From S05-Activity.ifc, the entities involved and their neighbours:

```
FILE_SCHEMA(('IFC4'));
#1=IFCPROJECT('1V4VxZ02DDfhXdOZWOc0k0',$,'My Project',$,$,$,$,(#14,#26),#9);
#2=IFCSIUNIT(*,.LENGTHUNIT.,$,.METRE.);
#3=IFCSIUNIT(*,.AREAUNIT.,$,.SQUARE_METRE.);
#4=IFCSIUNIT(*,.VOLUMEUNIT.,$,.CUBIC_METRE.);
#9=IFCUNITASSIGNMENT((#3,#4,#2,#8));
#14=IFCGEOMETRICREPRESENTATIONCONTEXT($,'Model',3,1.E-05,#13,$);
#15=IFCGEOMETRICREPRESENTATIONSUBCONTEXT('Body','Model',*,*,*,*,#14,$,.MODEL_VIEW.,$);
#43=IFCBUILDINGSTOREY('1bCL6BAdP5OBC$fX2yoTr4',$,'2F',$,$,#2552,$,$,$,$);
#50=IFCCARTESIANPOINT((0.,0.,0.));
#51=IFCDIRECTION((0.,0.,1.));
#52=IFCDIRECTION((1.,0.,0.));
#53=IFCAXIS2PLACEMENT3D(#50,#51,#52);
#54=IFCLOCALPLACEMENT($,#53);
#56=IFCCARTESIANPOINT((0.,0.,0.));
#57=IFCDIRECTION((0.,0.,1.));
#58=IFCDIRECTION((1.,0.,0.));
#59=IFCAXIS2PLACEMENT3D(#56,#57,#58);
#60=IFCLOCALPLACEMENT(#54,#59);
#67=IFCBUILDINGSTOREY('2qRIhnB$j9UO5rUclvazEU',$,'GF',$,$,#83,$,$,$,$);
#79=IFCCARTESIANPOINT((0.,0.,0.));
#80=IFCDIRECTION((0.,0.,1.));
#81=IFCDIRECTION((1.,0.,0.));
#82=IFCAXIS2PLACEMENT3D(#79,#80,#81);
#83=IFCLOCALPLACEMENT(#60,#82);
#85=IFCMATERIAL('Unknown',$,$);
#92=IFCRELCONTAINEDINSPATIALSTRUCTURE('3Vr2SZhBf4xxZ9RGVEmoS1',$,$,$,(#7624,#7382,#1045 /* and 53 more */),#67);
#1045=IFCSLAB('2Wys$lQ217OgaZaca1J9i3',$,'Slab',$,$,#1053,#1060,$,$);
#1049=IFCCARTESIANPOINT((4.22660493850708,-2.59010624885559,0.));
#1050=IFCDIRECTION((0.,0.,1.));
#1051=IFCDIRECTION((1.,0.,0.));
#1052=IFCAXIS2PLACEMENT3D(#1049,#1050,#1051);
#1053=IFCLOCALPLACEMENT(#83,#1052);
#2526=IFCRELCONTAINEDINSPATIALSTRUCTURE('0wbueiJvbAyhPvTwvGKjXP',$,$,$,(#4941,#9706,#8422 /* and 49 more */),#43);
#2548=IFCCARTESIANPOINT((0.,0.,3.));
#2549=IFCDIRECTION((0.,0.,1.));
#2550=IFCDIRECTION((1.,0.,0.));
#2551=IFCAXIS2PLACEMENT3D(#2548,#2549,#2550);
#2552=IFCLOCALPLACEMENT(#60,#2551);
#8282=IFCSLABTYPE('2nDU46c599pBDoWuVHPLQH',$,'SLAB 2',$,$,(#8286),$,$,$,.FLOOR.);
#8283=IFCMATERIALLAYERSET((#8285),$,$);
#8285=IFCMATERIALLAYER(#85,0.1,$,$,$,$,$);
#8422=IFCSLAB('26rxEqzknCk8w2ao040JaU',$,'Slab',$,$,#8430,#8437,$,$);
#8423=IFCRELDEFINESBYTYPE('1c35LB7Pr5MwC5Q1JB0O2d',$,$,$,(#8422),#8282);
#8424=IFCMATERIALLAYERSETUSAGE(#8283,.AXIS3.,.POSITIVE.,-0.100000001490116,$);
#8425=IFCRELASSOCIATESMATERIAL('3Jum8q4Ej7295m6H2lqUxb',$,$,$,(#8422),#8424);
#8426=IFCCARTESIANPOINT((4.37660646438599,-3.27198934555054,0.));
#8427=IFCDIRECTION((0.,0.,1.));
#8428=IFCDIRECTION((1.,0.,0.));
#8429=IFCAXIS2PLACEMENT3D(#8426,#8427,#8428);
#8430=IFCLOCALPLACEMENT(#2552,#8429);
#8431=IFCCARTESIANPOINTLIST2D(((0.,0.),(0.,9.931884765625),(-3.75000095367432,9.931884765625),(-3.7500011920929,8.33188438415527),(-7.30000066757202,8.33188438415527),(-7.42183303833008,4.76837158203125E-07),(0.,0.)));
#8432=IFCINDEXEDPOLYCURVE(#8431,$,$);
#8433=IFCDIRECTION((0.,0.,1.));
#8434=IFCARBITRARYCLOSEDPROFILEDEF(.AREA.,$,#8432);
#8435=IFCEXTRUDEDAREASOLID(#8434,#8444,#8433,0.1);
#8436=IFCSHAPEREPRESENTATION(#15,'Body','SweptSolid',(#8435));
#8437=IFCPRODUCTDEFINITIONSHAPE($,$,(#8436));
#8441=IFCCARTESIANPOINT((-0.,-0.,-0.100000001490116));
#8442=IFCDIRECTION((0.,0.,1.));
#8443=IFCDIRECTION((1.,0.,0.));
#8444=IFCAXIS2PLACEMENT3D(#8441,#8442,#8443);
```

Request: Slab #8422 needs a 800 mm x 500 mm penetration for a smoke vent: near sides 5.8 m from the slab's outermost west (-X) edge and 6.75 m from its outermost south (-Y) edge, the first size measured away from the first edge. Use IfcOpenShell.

```python
import numpy as np
import ifcopenshell
import ifcopenshell.api.feature
import ifcopenshell.api.geometry
import ifcopenshell.api.root
import ifcopenshell.geom
import ifcopenshell.util.placement
import ifcopenshell.util.representation
import ifcopenshell.util.shape
import ifcopenshell.util.unit

model = ifcopenshell.open("S05-Activity.ifc")
unit_scale = ifcopenshell.util.unit.calculate_unit_scale(model)
settings = ifcopenshell.geom.settings()


def volume(element):
    """Net volume in cubic metres, openings subtracted."""
    shape = ifcopenshell.geom.create_shape(settings, element)
    return ifcopenshell.util.shape.get_volume(shape.geometry)


slab = model.by_id(8422)
before = volume(slab)

# Extent in the slab's own axes, in metres. The edges named are its -X and -Y sides.
slab_shape = ifcopenshell.geom.create_shape(settings, slab)
vertices = ifcopenshell.util.shape.get_vertices(slab_shape.geometry)
x_min, y_min, bottom = vertices.min(axis=0)
top = vertices[:, 2].max()

opening = ifcopenshell.api.root.create_entity(model, ifc_class="IfcOpeningElement", name="Smoke vent opening", predefined_type="OPENING")
context = ifcopenshell.util.representation.get_context(model, "Model", "Body", "MODEL_VIEW")
width, depth = 0.8, 0.5
outline = [(0.0, 0.0), (width, 0.0), (width, depth), (0.0, depth), (0.0, 0.0)]
# Overshoot both faces by 50 mm so the cut is clean.
shape = ifcopenshell.api.geometry.add_slab_representation(
    model, context=context, depth=top - bottom + 0.1, polyline=outline
)
ifcopenshell.api.geometry.assign_representation(model, product=opening, representation=shape)

matrix = ifcopenshell.util.placement.get_local_placement(slab.ObjectPlacement)
matrix[:, 3] = matrix @ np.append(np.array([x_min + 5.8, y_min + 6.75, bottom - 0.05]) / unit_scale, 1.0)
ifcopenshell.api.geometry.edit_object_placement(model, product=opening, matrix=matrix, is_si=False)
ifcopenshell.api.feature.add_feature(model, feature=opening, element=slab)

after = volume(slab)

print(f"slab volume {before:.3f} -> {after:.3f} m3")

model.write("S05-Activity_v2.ifc")
```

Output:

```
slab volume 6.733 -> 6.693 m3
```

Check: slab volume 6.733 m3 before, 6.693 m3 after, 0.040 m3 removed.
